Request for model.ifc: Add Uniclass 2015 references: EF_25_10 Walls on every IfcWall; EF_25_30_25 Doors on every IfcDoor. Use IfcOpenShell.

First a look at what the model holds.

```python
import ifcopenshell

model = ifcopenshell.open("model.ifc")
print(model.schema)
print("classifications:", [c.Name for c in model.by_type("IfcClassification")])
for ifc_class in ("IfcDoor", "IfcRoof", "IfcStair", "IfcWall", "IfcWindow"):
    print(ifc_class, len(model.by_type(ifc_class)))
```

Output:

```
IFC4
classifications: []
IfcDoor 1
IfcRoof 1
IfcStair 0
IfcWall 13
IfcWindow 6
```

```python
import ifcopenshell
import ifcopenshell.api.classification

model = ifcopenshell.open("model.ifc")

system = ifcopenshell.api.classification.add_classification(model, classification="Uniclass 2015")

codes = {
    "IfcWall": ("EF_25_10", "Walls"),
    "IfcDoor": ("EF_25_30_25", "Doors"),
}
for ifc_class, (code, name) in codes.items():
    products = model.by_type(ifc_class)
    ifcopenshell.api.classification.add_reference(
        model, products=products, classification=system, identification=code, name=name
    )
    print(code, len(products))

model.write("model_updated.ifc")
```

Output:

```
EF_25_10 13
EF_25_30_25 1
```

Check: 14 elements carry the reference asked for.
